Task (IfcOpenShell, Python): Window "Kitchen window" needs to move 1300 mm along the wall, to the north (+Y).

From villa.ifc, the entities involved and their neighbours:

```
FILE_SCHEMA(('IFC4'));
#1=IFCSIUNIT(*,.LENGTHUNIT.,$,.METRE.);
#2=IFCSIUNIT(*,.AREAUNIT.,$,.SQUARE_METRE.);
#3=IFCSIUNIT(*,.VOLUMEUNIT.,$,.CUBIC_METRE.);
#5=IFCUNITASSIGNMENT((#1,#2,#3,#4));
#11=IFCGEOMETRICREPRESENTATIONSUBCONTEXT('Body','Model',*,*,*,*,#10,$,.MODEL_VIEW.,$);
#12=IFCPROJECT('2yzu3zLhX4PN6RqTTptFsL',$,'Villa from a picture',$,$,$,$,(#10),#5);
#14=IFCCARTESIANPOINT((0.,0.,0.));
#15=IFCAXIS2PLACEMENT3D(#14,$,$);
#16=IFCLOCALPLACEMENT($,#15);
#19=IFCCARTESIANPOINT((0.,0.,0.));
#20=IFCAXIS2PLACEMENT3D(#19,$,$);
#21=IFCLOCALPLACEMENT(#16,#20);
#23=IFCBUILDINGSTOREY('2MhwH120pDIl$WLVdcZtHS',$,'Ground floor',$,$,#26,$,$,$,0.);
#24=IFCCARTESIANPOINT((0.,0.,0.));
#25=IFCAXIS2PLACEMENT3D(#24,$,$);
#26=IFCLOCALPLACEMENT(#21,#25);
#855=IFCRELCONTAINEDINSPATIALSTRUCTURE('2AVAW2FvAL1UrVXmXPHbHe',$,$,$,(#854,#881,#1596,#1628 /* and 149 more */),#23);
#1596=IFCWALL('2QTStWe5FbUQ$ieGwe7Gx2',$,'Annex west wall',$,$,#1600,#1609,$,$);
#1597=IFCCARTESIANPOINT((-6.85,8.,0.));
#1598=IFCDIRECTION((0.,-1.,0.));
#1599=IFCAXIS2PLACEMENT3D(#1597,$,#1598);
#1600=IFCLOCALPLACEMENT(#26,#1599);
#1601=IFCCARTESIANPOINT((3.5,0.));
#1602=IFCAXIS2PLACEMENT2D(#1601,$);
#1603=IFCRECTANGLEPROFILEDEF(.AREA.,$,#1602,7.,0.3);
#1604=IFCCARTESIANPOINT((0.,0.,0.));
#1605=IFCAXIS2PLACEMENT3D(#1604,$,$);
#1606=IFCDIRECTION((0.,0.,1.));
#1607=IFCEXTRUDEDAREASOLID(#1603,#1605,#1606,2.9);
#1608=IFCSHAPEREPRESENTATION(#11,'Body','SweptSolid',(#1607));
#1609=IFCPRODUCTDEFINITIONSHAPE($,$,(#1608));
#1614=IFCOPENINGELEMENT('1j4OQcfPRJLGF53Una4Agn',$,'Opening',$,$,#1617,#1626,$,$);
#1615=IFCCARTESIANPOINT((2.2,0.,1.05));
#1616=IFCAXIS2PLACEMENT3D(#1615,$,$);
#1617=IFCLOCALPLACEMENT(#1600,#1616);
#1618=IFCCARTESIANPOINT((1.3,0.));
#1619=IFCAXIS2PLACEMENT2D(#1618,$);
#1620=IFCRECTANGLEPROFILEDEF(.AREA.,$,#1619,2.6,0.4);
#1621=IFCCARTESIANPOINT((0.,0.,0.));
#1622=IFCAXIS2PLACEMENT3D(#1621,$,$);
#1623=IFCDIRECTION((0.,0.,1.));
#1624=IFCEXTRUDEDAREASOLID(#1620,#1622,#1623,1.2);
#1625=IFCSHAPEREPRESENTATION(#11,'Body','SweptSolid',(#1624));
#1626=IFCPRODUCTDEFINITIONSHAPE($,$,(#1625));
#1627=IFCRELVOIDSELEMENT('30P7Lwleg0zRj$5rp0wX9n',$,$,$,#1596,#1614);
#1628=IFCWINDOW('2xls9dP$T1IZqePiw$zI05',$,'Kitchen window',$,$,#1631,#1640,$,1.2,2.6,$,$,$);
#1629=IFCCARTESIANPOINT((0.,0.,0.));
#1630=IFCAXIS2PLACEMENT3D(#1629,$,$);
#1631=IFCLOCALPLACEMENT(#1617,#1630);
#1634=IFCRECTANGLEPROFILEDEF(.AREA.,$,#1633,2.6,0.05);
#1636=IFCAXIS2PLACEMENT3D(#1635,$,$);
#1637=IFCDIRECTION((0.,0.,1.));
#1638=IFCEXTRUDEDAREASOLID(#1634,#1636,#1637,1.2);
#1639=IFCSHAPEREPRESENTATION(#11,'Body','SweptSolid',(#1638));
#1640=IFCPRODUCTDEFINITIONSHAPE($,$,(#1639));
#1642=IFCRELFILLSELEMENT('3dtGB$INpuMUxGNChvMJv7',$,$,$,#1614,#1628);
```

```python
import ifcopenshell
import ifcopenshell.api.geometry
import ifcopenshell.util.placement

model = ifcopenshell.open("villa.ifc")

window = model.by_guid("2xls9dP$T1IZqePiw$zI05")
opening = window.FillsVoids[0].RelatingOpeningElement
wall = opening.VoidsElements[0].RelatingBuildingElement

wall_matrix = ifcopenshell.util.placement.get_local_placement(wall.ObjectPlacement)
shift = wall_matrix[:3, 0] * -1.3
before = ifcopenshell.util.placement.get_local_placement(window.ObjectPlacement)[:3, 3].copy()

# The window is placed relative to its opening, so it follows when the opening moves.
matrix = ifcopenshell.util.placement.get_local_placement(opening.ObjectPlacement)
matrix[:3, 3] += shift
ifcopenshell.api.geometry.edit_object_placement(
    model, product=opening, matrix=matrix, is_si=False, should_transform_children=True
)

after = ifcopenshell.util.placement.get_local_placement(window.ObjectPlacement)[:3, 3]
print("window moved by", (after - before).round(3) + 0.0)

model.write("villa-out.ifc")
```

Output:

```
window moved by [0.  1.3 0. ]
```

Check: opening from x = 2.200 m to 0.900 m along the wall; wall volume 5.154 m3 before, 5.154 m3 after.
